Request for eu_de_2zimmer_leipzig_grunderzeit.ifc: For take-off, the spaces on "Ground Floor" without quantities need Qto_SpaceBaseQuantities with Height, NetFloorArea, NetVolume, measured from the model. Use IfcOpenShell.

First a look at what the model holds.

```python
import ifcopenshell
import ifcopenshell.util.element
import ifcopenshell.util.unit

model = ifcopenshell.open("eu_de_2zimmer_leipzig_grunderzeit.ifc")
print(model.schema)
for unit_type in ("LENGTHUNIT", "AREAUNIT", "VOLUMEUNIT"):
    print(unit_type, ifcopenshell.util.unit.calculate_unit_scale(model, unit_type))
storey = next(s for s in model.by_type("IfcBuildingStorey") if s.Name == "Ground Floor")
spaces = [e for e in ifcopenshell.util.element.get_decomposition(storey) if e.is_a("IfcSpace")]
for e in sorted(spaces, key=lambda e: e.id()):
    print(e.id(), e.is_a(), e.Name, list(ifcopenshell.util.element.get_psets(e, qtos_only=True)), sep=" | ")
```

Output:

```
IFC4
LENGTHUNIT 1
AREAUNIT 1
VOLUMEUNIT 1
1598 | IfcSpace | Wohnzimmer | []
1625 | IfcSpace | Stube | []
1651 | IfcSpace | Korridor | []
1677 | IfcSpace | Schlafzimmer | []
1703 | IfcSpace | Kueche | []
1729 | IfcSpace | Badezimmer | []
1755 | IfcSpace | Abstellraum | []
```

```python
import ifcopenshell
import ifcopenshell.api.pset
import ifcopenshell.geom
import ifcopenshell.util.element
import ifcopenshell.util.shape
import ifcopenshell.util.unit

model = ifcopenshell.open("eu_de_2zimmer_leipzig_grunderzeit.ifc")
unit_scale = ifcopenshell.util.unit.calculate_unit_scale(model)
area_scale = ifcopenshell.util.unit.calculate_unit_scale(model, "AREAUNIT")
volume_scale = ifcopenshell.util.unit.calculate_unit_scale(model, "VOLUMEUNIT")
settings = ifcopenshell.geom.settings()

storey = next(s for s in model.by_type("IfcBuildingStorey") if s.Name == "Ground Floor")
spaces = [e for e in ifcopenshell.util.element.get_decomposition(storey) if e.is_a("IfcSpace")]

for e in sorted(spaces, key=lambda e: e.id()):
    if ifcopenshell.util.element.get_psets(e, qtos_only=True, should_inherit=False):
        continue
    # Geometry comes back in metres, in the element's own axes.
    shape = ifcopenshell.geom.create_shape(settings, e)
    values = {
        "Height": ifcopenshell.util.shape.get_z(shape.geometry) / unit_scale,
        "NetFloorArea": ifcopenshell.util.shape.get_footprint_area(shape.geometry) / area_scale,
        "NetVolume": ifcopenshell.util.shape.get_volume(shape.geometry) / volume_scale,
    }
    qto = ifcopenshell.api.pset.add_qto(model, product=e, name="Qto_SpaceBaseQuantities")
    ifcopenshell.api.pset.edit_qto(model, qto=qto, properties=values)
    print(e.id(), {k: round(v, 3) for k, v in values.items()})

model.write("eu_de_2zimmer_leipzig_grunderzeit_v2.ifc")
```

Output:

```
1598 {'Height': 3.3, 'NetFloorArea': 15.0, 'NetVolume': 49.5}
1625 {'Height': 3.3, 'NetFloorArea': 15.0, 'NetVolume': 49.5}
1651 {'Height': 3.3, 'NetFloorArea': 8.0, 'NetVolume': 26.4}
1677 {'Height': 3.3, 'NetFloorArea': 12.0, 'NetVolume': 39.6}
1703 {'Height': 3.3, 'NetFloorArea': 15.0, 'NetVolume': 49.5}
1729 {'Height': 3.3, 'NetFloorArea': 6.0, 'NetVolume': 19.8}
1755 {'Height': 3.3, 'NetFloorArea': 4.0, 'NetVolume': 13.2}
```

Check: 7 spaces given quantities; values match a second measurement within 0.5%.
